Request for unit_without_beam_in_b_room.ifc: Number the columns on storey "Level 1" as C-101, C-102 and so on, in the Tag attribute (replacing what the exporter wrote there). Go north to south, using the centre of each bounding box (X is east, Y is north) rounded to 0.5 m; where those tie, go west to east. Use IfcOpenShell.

First a look at what the model holds.

```python
import ifcopenshell
import ifcopenshell.util.element
import ifcopenshell.util.placement

model = ifcopenshell.open("unit_without_beam_in_b_room.ifc")
print(model.schema)
storey = next(s for s in model.by_type("IfcBuildingStorey") if s.Name == "Level 1")
columns = [e for e in ifcopenshell.util.element.get_decomposition(storey) if e.is_a("IfcColumn")]
for e in sorted(columns, key=lambda e: e.id()):
    origin = ifcopenshell.util.placement.get_local_placement(e.ObjectPlacement)[:3, 3]
    print(e.id(), e.Tag, e.Name, origin.round(2) + 0.0, sep=" | ")
```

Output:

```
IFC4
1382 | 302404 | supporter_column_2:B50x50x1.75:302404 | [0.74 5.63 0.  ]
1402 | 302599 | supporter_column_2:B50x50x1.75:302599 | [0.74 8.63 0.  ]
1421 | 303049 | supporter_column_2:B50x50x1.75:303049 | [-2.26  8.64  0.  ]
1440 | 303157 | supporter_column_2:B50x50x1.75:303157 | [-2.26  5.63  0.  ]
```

```python
import ifcopenshell
import ifcopenshell.geom
import ifcopenshell.util.element
import ifcopenshell.util.shape

model = ifcopenshell.open("unit_without_beam_in_b_room.ifc")
settings = ifcopenshell.geom.settings()
settings.set("use-world-coords", True)


def centre(element):
    shape = ifcopenshell.geom.create_shape(settings, element)
    return ifcopenshell.util.shape.get_bbox_centroid(shape.geometry)


storey = next(s for s in model.by_type("IfcBuildingStorey") if s.Name == "Level 1")
columns = [e for e in ifcopenshell.util.element.get_decomposition(storey) if e.is_a("IfcColumn")]

# Insertion points can sit at a corner or the storey origin, so sort by the geometry (in metres).
centres = {e: centre(e) for e in columns}
columns.sort(key=lambda e: (-round(centres[e][1] / 0.5), centres[e][0]))

for i, e in enumerate(columns, start=1):
    number = f"C-1{i:02d}"
    e.Tag = number
    print(e.id(), number)

model.write("unit_without_beam_in_b_room-out.ifc")
```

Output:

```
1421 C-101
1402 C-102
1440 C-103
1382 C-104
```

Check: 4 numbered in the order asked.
